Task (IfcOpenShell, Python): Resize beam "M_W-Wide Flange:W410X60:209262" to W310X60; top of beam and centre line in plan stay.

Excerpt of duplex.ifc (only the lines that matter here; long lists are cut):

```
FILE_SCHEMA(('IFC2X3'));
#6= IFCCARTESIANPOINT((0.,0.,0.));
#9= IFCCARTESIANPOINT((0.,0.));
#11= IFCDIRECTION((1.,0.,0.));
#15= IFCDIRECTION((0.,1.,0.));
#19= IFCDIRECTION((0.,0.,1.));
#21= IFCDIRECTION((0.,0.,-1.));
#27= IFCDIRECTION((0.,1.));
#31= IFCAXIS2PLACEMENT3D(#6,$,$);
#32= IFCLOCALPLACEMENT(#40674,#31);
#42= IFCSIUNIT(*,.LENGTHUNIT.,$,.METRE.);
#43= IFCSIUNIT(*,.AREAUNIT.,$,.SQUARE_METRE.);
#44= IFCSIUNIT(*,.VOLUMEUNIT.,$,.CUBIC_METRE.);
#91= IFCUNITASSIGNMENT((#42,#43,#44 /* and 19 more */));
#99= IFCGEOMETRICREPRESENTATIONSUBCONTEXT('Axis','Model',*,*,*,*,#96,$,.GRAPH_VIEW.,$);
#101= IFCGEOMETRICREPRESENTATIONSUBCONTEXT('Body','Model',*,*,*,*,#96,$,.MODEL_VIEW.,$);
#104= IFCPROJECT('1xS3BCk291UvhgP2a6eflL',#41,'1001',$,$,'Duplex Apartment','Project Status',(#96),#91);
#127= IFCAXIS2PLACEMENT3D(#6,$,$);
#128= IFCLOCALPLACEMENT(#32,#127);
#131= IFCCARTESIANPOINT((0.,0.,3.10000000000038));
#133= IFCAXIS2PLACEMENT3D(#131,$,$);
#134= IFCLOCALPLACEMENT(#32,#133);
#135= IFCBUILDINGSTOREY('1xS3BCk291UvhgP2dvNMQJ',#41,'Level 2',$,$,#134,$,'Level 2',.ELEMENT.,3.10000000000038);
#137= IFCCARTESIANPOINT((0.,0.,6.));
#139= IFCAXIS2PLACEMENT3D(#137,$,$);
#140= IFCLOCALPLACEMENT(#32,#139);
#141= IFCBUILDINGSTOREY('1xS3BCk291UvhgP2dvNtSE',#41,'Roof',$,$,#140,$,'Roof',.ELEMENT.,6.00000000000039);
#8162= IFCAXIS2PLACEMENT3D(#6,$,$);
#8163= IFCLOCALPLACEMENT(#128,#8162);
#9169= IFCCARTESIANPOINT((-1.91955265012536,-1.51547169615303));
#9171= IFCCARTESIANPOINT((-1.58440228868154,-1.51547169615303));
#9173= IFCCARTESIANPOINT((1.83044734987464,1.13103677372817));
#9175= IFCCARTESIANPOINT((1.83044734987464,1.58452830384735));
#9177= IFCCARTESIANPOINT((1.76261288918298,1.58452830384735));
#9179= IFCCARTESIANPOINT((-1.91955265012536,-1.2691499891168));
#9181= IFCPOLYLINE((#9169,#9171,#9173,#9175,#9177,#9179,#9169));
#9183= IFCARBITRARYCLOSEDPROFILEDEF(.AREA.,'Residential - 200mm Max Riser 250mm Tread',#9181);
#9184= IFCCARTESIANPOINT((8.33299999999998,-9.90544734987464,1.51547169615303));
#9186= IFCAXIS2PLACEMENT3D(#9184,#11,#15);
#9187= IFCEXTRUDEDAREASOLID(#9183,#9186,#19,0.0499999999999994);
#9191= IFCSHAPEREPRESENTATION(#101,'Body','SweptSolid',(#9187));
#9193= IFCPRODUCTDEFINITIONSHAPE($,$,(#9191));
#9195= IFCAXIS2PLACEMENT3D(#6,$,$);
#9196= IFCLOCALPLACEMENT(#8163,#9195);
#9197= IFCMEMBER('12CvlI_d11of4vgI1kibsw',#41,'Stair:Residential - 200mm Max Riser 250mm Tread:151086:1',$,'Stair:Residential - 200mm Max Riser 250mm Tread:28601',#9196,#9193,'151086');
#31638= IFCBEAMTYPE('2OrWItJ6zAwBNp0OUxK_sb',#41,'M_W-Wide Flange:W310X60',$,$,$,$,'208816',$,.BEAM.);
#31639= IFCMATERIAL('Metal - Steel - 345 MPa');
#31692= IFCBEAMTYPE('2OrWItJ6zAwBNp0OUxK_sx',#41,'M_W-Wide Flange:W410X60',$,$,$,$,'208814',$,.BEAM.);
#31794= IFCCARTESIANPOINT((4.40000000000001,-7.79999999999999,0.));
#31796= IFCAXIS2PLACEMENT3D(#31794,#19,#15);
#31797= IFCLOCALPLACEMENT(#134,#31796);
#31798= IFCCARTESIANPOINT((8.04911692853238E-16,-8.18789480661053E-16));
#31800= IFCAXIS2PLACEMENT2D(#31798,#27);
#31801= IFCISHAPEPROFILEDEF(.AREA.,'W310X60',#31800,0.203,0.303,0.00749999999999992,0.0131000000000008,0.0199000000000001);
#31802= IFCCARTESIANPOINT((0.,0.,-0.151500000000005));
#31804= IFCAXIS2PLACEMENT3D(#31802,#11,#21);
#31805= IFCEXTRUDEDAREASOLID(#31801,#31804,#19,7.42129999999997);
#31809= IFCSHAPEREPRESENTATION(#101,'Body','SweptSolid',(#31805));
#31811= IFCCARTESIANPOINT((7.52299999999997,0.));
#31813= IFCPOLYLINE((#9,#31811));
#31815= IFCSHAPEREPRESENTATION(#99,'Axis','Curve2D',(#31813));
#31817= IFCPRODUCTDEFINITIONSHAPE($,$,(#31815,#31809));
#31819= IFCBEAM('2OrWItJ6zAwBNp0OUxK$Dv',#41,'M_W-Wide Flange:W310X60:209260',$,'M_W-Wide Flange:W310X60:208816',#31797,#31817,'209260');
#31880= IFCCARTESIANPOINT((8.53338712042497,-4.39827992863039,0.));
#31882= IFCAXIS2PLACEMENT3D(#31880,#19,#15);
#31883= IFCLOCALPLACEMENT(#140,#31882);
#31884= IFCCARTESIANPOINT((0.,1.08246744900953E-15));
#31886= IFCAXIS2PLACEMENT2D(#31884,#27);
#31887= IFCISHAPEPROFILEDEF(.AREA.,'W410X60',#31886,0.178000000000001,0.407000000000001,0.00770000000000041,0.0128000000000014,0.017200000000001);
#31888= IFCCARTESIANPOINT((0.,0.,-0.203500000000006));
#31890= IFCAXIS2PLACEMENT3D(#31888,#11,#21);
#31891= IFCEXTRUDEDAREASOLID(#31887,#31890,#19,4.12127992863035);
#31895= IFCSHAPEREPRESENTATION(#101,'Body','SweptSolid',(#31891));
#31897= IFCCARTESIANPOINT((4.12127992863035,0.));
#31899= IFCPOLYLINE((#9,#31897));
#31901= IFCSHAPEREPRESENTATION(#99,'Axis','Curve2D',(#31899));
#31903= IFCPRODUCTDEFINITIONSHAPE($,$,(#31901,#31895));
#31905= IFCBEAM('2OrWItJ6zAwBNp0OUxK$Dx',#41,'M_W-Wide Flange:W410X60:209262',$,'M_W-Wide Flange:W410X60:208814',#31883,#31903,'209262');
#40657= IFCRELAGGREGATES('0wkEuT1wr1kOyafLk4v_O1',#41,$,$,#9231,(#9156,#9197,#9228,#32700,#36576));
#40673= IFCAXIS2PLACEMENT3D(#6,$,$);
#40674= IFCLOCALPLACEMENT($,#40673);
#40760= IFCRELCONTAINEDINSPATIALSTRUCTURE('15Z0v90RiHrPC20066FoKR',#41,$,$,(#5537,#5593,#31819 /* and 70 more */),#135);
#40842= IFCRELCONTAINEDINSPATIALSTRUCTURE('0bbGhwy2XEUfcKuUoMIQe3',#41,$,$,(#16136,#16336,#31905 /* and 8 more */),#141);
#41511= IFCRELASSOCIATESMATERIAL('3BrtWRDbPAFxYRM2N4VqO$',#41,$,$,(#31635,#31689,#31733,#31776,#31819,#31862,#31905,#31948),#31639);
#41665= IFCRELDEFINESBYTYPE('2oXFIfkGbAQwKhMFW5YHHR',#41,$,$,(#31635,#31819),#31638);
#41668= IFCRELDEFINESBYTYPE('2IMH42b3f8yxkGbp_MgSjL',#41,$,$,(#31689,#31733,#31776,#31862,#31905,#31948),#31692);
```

```python
import ifcopenshell
import ifcopenshell.api.type
import ifcopenshell.util.element
import ifcopenshell.util.representation

model = ifcopenshell.open("duplex.ifc")

member = model.by_guid("2OrWItJ6zAwBNp0OUxK$Dx")
source = next(p for p in model.by_type("IfcIShapeProfileDef") if p.ProfileName == "W310X60")

body = ifcopenshell.util.representation.get_representation(member, "Model", "Body")
solid = body.Items[0]
old_profile = solid.SweptArea

# Copy the section's sizes but keep this member's own profile position.
profile = ifcopenshell.util.element.copy(model, source)
# Profiles are centred, so shift by half the change in depth to hold the top.
shift = (old_profile.OverallDepth - profile.OverallDepth) / 2
x, y = old_profile.Position.Location.Coordinates
up = (-1.0, 0.0)  # upwards, in the solid's own plane
location = model.createIfcCartesianPoint((x + up[0] * shift, y + up[1] * shift))
profile.Position = model.createIfcAxis2Placement2D(location, old_profile.Position.RefDirection)
solid.SweptArea = profile
if not model.get_total_inverses(old_profile):
    ifcopenshell.util.element.remove_deep2(model, old_profile)

new_type = model.by_id(31638)
ifcopenshell.api.type.assign_type(
    model, related_objects=[member], relating_type=new_type, should_map_representations=False
)
member.Name = member.Name.replace("W410X60", "W310X60")
member.ObjectType = "M_W-Wide Flange:W310X60:208814"

print(solid.SweptArea)

model.write("duplex_rev.ifc")
```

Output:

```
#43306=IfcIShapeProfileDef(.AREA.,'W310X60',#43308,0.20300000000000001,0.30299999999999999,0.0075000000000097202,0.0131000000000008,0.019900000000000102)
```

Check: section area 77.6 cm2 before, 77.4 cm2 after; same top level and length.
